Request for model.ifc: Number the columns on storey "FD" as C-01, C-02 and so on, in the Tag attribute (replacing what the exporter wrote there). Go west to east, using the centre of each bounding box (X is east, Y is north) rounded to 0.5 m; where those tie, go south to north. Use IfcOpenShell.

First a look at what the model holds.

```python
import ifcopenshell
import ifcopenshell.util.element
import ifcopenshell.util.placement

model = ifcopenshell.open("model.ifc")
print(model.schema)
storey = next(s for s in model.by_type("IfcBuildingStorey") if s.Name == "FD")
columns = [e for e in ifcopenshell.util.element.get_decomposition(storey) if e.is_a("IfcColumn")]
for e in sorted(columns, key=lambda e: e.id()):
    origin = ifcopenshell.util.placement.get_local_placement(e.ObjectPlacement)[:3, 3]
    print(e.id(), e.Tag, e.Name, origin.round(2) + 0.0, sep=" | ")
```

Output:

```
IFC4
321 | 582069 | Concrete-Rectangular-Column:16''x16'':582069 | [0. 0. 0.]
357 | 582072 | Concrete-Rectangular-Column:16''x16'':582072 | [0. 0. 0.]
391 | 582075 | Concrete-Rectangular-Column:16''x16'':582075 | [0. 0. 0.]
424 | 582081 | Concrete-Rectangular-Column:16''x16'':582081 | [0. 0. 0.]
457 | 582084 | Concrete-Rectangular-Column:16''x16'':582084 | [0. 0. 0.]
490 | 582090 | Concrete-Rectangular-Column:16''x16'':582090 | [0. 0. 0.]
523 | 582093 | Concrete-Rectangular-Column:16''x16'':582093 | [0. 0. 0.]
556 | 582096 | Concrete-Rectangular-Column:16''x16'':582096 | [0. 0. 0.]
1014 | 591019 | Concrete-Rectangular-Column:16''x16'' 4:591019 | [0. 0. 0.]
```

```python
import ifcopenshell
import ifcopenshell.geom
import ifcopenshell.util.element
import ifcopenshell.util.shape

model = ifcopenshell.open("model.ifc")
settings = ifcopenshell.geom.settings()
settings.set("use-world-coords", True)


def centre(element):
    shape = ifcopenshell.geom.create_shape(settings, element)
    return ifcopenshell.util.shape.get_bbox_centroid(shape.geometry)


storey = next(s for s in model.by_type("IfcBuildingStorey") if s.Name == "FD")
columns = [e for e in ifcopenshell.util.element.get_decomposition(storey) if e.is_a("IfcColumn")]

# Insertion points can sit at a corner or the storey origin, so sort by the geometry (in metres).
centres = {e: centre(e) for e in columns}
columns.sort(key=lambda e: (round(centres[e][0] / 0.5), centres[e][1]))

for i, e in enumerate(columns, start=1):
    number = f"C-{i:02d}"
    e.Tag = number
    print(e.id(), number)

model.write("model-out.ifc")
```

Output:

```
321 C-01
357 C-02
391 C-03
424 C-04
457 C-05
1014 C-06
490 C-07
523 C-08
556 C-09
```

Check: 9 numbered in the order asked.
